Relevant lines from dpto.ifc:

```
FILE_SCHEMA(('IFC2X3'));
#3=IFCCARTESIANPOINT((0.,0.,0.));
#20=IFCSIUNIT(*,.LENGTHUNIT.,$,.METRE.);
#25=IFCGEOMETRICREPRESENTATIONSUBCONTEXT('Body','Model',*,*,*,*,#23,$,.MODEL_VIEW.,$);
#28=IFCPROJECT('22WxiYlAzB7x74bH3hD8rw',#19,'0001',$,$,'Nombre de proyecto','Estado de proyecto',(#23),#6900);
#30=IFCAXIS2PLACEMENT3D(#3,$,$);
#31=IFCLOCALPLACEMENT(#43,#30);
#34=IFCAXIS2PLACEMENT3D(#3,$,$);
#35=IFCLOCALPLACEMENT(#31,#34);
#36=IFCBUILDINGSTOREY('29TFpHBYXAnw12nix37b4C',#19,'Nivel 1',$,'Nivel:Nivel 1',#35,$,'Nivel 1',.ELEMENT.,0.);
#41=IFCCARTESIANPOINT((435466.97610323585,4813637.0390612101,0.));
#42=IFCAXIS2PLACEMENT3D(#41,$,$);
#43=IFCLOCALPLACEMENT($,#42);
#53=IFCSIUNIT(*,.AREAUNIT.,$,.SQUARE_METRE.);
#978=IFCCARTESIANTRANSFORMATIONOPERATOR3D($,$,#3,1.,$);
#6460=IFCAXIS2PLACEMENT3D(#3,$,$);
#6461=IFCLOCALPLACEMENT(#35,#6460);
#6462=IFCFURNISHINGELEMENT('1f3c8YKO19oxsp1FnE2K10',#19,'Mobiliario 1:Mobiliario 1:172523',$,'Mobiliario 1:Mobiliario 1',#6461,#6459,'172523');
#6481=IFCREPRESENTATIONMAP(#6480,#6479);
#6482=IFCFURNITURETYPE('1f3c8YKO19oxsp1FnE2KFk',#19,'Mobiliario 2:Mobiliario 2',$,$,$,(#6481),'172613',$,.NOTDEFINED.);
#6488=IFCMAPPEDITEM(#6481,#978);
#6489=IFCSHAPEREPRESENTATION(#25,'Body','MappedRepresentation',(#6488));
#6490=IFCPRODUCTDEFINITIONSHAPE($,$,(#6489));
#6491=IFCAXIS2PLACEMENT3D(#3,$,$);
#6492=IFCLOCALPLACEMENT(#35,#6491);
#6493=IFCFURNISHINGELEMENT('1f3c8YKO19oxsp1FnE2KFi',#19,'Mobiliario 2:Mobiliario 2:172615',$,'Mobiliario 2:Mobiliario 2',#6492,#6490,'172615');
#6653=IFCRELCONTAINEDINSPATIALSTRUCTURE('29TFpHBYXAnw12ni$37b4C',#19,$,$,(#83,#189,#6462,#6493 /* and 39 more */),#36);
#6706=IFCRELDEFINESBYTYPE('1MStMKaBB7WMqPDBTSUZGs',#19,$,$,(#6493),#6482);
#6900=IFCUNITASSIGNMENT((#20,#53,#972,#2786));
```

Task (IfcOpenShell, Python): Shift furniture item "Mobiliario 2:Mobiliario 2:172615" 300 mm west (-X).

```python
import ifcopenshell
import ifcopenshell.api.geometry
import ifcopenshell.util.placement
import ifcopenshell.util.unit

model = ifcopenshell.open("dpto.ifc")
unit_scale = ifcopenshell.util.unit.calculate_unit_scale(model)

item = model.by_guid("1f3c8YKO19oxsp1FnE2KFi")
matrix = ifcopenshell.util.placement.get_local_placement(item.ObjectPlacement)
matrix[0, 3] -= 0.3 / unit_scale
ifcopenshell.api.geometry.edit_object_placement(model, product=item, matrix=matrix, is_si=False)

print(ifcopenshell.util.placement.get_local_placement(item.ObjectPlacement).round(3) + 0.0)

model.write("dpto_rev.ifc")
```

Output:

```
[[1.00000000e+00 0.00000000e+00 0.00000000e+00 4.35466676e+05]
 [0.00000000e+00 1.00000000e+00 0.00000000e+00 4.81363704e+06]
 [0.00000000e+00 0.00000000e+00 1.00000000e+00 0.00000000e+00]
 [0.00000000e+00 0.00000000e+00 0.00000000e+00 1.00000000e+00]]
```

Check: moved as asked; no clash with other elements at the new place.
